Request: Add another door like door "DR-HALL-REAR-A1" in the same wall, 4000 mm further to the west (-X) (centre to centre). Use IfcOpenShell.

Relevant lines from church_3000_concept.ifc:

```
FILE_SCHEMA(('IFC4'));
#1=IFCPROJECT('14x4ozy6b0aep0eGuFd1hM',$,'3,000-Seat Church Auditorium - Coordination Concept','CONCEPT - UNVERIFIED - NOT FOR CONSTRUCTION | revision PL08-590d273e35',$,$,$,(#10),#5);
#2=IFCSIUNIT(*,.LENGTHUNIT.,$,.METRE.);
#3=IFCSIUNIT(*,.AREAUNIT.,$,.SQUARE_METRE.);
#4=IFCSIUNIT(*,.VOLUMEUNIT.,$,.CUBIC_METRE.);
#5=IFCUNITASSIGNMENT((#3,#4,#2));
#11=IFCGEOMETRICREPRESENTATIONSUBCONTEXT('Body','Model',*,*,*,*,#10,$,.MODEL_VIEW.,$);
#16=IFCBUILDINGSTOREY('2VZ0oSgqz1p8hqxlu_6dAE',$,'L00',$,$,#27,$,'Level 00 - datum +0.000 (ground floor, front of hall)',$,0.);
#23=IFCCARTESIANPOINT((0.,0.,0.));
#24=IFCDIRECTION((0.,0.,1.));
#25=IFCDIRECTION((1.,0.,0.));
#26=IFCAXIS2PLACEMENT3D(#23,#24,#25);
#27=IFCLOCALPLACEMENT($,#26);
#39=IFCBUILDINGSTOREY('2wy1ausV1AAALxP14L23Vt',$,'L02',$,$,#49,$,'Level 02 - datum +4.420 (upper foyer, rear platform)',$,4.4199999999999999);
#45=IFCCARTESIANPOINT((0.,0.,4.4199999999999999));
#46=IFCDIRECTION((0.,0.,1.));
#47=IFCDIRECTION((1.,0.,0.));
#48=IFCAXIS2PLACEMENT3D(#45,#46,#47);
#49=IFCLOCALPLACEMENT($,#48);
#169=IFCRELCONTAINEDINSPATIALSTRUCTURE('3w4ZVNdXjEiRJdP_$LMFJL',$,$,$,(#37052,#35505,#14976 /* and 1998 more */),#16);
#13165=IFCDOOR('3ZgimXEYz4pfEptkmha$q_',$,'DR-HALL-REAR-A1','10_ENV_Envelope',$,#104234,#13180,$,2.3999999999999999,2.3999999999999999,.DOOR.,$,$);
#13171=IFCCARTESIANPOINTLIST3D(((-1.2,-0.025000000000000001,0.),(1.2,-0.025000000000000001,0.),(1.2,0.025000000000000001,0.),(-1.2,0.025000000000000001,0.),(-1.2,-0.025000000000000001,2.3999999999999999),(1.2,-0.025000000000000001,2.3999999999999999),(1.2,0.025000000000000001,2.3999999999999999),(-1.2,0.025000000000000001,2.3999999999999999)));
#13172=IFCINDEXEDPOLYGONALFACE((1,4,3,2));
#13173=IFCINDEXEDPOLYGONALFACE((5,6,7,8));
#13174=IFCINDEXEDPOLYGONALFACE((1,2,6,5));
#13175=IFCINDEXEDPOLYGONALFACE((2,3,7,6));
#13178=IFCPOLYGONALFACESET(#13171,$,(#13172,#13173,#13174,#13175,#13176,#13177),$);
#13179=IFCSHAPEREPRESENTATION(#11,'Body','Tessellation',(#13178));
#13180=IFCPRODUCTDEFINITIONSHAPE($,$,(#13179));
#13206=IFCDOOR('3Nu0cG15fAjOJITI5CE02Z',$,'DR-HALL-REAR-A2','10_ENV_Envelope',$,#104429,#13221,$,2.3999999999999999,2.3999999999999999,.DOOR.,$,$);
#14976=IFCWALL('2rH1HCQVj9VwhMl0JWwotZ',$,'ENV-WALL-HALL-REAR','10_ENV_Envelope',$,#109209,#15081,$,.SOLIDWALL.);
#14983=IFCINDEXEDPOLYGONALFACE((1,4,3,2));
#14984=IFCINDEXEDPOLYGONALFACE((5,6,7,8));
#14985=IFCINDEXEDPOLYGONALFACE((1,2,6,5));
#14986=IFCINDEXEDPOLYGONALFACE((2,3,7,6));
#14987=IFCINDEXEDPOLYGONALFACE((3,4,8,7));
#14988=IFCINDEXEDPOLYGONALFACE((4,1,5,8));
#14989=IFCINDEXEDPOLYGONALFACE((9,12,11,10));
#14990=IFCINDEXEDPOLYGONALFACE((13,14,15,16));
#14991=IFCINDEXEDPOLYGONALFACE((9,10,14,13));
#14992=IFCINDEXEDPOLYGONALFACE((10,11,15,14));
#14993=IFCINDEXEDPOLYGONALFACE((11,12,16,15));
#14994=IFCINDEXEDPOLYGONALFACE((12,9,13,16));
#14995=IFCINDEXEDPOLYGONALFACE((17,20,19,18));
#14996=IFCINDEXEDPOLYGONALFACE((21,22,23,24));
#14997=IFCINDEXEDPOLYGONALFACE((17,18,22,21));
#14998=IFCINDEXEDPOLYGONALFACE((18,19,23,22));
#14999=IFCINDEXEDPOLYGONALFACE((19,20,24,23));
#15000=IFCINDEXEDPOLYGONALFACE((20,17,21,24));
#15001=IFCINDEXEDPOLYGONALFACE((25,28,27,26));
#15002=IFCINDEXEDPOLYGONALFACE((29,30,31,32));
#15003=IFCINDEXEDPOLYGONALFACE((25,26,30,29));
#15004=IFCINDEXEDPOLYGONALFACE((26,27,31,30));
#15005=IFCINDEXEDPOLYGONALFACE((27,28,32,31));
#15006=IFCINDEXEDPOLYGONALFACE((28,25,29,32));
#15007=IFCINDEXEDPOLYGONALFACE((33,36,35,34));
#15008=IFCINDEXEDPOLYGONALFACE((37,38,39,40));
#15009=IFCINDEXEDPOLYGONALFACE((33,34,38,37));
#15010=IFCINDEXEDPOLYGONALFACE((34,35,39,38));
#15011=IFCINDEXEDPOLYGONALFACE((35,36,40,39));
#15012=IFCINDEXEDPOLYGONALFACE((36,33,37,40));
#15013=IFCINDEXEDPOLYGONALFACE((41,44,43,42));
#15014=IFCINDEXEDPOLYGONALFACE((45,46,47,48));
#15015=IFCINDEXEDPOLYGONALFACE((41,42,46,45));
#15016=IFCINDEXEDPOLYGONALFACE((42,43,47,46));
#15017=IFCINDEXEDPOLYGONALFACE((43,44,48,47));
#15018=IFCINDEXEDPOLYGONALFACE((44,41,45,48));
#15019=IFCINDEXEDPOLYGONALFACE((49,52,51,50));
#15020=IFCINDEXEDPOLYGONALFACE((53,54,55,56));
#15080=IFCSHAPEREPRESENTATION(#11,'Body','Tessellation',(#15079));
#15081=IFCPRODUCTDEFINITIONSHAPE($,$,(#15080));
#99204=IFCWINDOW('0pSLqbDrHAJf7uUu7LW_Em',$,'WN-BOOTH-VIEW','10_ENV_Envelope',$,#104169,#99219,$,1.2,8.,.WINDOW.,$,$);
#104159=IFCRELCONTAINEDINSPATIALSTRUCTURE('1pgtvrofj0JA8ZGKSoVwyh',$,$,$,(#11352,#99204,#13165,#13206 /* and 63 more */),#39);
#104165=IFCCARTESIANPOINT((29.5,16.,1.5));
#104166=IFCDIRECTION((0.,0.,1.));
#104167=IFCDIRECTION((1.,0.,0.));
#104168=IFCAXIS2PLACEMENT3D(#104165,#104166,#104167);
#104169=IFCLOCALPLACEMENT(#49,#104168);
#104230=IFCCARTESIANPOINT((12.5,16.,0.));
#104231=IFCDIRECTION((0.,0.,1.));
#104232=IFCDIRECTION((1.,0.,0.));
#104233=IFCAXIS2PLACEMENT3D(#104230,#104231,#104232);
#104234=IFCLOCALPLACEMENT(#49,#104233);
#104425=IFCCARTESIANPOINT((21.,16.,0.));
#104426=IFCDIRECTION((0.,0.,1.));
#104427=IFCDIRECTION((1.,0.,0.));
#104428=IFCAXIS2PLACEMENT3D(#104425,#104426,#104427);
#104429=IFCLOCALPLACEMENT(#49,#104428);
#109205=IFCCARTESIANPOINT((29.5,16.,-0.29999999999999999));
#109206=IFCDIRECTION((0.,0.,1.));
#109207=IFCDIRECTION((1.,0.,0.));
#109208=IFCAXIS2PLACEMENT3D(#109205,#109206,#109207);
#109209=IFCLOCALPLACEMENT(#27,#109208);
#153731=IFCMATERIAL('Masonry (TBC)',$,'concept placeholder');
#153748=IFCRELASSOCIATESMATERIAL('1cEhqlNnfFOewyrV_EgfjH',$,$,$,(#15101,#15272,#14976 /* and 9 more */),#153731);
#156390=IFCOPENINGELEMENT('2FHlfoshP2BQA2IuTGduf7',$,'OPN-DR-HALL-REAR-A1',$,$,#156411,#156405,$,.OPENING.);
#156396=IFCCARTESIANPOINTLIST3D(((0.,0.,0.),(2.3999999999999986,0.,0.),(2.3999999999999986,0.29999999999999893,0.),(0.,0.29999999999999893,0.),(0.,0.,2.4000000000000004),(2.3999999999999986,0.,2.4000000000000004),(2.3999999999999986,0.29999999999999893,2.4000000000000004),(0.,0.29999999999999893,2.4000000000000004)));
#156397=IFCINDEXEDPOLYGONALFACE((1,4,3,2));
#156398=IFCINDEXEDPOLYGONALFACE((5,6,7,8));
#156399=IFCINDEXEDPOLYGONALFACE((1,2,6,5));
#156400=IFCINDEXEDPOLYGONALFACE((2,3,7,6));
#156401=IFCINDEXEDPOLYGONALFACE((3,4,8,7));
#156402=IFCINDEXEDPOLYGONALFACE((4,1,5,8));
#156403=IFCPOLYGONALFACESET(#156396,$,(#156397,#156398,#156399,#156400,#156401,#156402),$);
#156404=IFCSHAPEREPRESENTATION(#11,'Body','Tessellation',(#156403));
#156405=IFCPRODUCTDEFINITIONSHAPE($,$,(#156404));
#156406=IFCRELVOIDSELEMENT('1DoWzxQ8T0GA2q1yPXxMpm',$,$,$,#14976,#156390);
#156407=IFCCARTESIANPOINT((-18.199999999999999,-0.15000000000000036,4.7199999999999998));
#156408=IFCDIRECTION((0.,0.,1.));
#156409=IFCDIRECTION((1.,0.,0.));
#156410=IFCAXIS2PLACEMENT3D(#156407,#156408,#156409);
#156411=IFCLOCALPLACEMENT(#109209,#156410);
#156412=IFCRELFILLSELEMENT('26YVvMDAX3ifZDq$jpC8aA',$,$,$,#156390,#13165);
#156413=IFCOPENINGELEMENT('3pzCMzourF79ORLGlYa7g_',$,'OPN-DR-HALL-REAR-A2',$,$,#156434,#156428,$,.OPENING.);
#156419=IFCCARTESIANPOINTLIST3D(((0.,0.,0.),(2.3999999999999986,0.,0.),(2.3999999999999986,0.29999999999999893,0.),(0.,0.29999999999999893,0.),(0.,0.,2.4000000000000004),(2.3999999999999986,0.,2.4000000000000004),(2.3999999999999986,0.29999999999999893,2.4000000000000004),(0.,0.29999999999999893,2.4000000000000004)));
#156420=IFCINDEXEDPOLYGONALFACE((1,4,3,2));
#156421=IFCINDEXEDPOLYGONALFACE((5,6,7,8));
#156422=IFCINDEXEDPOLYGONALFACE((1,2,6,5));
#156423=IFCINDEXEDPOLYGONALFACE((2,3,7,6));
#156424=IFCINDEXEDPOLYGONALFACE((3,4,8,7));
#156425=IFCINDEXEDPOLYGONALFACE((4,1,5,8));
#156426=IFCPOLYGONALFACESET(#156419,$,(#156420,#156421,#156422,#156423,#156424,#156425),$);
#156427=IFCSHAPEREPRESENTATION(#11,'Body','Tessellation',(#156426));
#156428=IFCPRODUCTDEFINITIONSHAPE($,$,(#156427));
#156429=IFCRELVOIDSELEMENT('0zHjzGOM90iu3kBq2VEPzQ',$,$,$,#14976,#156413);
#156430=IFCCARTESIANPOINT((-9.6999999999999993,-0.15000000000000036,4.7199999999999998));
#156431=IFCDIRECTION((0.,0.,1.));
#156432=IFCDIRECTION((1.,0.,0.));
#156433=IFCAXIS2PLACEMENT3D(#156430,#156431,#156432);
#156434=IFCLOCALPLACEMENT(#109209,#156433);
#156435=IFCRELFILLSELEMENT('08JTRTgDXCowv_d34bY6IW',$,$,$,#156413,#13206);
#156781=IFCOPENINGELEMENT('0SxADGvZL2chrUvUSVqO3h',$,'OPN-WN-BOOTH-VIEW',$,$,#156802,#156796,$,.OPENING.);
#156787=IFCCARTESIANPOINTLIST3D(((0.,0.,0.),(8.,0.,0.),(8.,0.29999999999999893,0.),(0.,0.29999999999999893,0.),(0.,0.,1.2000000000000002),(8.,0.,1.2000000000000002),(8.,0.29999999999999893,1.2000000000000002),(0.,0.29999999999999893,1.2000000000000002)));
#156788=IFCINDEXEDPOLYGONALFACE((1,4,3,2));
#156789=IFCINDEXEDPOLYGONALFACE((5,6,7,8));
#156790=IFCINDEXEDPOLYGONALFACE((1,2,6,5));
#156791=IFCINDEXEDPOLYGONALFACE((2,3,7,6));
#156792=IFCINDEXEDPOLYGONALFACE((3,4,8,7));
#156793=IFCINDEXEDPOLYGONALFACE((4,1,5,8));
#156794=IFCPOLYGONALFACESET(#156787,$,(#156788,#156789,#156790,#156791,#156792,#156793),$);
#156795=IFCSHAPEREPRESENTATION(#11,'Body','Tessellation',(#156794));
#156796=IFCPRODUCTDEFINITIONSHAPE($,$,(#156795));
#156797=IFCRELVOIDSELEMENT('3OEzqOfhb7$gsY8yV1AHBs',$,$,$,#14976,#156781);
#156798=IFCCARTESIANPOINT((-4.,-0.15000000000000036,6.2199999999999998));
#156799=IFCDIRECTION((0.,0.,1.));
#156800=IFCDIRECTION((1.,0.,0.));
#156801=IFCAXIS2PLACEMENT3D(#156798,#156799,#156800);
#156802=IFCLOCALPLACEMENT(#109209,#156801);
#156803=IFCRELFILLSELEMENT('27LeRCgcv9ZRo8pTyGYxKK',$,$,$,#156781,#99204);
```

```python
import ifcopenshell
import ifcopenshell.api.feature
import ifcopenshell.api.geometry
import ifcopenshell.api.root
import ifcopenshell.geom
import ifcopenshell.util.element
import ifcopenshell.util.placement
import ifcopenshell.util.shape

model = ifcopenshell.open("church_3000_concept.ifc")
settings = ifcopenshell.geom.settings()


def volume(element):
    """Net volume in cubic metres, openings subtracted."""
    shape = ifcopenshell.geom.create_shape(settings, element)
    return ifcopenshell.util.shape.get_volume(shape.geometry)


door = model.by_guid("3ZgimXEYz4pfEptkmha$q_")
opening = door.FillsVoids[0].RelatingOpeningElement
wall = opening.VoidsElements[0].RelatingBuildingElement
before = volume(wall)
shift = ifcopenshell.util.placement.get_local_placement(wall.ObjectPlacement)[:3, 0] * -4.0

# copy_class copies the void relationship, type, container and properties, but no geometry.
new_opening = ifcopenshell.api.root.copy_class(model, product=opening)
new_opening.Representation = ifcopenshell.util.element.copy_deep(
    model, opening.Representation, exclude=["IfcGeometricRepresentationContext", "IfcRepresentationMap"]
)
new_door = ifcopenshell.api.root.copy_class(model, product=door)
new_door.Representation = ifcopenshell.util.element.copy_deep(
    model, door.Representation, exclude=["IfcGeometricRepresentationContext", "IfcRepresentationMap"]
)
ifcopenshell.api.feature.add_filling(model, opening=new_opening, element=new_door)

for old, new in ((opening, new_opening), (door, new_door)):
    matrix = ifcopenshell.util.placement.get_local_placement(old.ObjectPlacement)
    matrix[:3, 3] += shift
    ifcopenshell.api.geometry.edit_object_placement(model, product=new, matrix=matrix, is_si=False)

after = volume(wall)

print(f"wall volume {before:.3f} -> {after:.3f} m3")

model.write("church_3000_concept-out.ifc")
```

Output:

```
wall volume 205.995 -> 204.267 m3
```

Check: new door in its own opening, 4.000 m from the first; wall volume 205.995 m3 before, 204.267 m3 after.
